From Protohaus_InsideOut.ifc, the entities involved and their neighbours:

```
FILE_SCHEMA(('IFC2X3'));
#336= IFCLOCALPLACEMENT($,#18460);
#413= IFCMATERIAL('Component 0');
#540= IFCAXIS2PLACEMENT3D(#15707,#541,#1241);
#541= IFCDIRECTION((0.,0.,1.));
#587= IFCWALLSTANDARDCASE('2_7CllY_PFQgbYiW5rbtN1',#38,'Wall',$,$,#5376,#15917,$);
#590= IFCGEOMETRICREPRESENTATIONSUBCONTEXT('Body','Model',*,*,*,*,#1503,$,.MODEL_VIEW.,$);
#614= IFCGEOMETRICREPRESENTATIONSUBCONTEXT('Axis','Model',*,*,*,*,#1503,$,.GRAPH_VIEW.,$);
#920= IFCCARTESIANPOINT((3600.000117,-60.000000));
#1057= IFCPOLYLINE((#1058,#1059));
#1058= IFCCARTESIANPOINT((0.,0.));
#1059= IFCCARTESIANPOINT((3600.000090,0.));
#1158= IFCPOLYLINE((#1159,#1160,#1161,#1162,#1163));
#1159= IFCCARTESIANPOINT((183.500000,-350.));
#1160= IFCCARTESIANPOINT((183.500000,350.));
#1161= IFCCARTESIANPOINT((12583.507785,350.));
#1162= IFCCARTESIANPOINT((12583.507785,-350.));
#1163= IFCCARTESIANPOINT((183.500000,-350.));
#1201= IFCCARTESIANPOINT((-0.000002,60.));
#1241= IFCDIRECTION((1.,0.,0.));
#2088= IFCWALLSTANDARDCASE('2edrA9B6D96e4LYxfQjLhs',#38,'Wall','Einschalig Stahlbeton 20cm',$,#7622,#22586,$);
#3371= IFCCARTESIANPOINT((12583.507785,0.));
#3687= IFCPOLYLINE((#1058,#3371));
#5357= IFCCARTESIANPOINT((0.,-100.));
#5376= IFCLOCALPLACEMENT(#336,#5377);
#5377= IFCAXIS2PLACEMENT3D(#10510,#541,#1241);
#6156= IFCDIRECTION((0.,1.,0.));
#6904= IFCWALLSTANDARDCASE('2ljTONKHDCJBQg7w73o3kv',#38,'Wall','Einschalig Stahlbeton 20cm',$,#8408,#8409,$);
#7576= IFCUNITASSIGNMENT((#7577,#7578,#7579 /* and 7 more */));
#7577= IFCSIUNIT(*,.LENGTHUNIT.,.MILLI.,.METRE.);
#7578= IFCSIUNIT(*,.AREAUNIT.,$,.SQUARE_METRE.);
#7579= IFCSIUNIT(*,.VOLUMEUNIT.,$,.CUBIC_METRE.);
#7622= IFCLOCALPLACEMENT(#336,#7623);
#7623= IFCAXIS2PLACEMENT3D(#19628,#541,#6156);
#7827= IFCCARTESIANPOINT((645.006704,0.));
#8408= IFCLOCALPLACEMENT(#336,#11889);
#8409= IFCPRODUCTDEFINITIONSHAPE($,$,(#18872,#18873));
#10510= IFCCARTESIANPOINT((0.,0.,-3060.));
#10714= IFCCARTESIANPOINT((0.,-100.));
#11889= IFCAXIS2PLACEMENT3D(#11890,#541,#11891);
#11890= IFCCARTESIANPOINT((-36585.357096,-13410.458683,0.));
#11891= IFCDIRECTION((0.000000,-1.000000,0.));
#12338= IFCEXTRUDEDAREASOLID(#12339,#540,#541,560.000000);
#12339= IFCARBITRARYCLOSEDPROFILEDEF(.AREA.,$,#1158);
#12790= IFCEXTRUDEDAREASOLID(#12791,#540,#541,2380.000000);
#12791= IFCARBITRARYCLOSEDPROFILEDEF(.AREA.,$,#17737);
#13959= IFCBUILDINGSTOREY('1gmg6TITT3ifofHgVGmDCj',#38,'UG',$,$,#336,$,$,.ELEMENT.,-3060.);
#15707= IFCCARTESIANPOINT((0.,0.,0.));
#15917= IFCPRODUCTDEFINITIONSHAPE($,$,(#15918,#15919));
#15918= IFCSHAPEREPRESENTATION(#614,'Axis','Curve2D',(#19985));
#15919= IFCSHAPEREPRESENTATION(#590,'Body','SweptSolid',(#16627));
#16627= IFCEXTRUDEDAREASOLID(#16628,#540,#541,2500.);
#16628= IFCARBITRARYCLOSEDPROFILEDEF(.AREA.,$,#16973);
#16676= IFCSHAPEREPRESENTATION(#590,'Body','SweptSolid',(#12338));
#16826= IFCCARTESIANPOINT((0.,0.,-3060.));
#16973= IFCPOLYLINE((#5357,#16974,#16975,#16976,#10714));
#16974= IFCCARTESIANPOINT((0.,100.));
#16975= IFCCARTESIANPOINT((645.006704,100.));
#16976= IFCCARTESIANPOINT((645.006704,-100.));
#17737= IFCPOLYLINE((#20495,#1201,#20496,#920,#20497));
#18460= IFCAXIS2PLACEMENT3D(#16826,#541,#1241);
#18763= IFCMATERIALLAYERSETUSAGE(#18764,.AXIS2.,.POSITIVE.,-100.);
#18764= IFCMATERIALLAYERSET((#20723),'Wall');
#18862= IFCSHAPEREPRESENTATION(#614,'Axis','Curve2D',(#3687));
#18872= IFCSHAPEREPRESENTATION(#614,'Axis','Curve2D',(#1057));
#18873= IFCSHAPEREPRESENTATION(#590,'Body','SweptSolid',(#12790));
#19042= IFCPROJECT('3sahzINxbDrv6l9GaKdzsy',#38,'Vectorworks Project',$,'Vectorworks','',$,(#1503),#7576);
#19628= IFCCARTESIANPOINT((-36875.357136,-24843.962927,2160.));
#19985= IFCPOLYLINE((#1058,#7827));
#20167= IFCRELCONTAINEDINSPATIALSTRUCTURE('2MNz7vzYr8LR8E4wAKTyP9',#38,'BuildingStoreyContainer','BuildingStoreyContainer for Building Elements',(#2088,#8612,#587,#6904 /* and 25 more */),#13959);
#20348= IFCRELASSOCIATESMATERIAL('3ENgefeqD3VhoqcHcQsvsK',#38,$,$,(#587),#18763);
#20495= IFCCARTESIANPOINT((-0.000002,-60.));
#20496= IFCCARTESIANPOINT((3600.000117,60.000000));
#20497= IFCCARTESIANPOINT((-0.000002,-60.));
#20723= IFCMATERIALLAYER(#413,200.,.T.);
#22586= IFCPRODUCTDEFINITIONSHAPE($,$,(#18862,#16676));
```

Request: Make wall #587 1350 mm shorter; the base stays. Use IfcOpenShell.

```python
import ifcopenshell
import ifcopenshell.geom
import ifcopenshell.util.representation
import ifcopenshell.util.shape
import ifcopenshell.util.unit

model = ifcopenshell.open("Protohaus_InsideOut.ifc")
unit_scale = ifcopenshell.util.unit.calculate_unit_scale(model)
settings = ifcopenshell.geom.settings()


def volume(element):
    """Net volume in cubic metres, openings subtracted."""
    shape = ifcopenshell.geom.create_shape(settings, element)
    return ifcopenshell.util.shape.get_volume(shape.geometry)


wall = model.by_id(587)
before = volume(wall)

body = ifcopenshell.util.representation.get_representation(wall, "Model", "Body")
solid = body.Items[0]
old_height = solid.Depth
solid.Depth -= 1.35 / unit_scale
after = volume(wall)

print(f"height {old_height:g} -> {solid.Depth:g}, volume {before:.3f} -> {after:.3f} m3")

model.write("Protohaus_InsideOut_rev.ifc")
```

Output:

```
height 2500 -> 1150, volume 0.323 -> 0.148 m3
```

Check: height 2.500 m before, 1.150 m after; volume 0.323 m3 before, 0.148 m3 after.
